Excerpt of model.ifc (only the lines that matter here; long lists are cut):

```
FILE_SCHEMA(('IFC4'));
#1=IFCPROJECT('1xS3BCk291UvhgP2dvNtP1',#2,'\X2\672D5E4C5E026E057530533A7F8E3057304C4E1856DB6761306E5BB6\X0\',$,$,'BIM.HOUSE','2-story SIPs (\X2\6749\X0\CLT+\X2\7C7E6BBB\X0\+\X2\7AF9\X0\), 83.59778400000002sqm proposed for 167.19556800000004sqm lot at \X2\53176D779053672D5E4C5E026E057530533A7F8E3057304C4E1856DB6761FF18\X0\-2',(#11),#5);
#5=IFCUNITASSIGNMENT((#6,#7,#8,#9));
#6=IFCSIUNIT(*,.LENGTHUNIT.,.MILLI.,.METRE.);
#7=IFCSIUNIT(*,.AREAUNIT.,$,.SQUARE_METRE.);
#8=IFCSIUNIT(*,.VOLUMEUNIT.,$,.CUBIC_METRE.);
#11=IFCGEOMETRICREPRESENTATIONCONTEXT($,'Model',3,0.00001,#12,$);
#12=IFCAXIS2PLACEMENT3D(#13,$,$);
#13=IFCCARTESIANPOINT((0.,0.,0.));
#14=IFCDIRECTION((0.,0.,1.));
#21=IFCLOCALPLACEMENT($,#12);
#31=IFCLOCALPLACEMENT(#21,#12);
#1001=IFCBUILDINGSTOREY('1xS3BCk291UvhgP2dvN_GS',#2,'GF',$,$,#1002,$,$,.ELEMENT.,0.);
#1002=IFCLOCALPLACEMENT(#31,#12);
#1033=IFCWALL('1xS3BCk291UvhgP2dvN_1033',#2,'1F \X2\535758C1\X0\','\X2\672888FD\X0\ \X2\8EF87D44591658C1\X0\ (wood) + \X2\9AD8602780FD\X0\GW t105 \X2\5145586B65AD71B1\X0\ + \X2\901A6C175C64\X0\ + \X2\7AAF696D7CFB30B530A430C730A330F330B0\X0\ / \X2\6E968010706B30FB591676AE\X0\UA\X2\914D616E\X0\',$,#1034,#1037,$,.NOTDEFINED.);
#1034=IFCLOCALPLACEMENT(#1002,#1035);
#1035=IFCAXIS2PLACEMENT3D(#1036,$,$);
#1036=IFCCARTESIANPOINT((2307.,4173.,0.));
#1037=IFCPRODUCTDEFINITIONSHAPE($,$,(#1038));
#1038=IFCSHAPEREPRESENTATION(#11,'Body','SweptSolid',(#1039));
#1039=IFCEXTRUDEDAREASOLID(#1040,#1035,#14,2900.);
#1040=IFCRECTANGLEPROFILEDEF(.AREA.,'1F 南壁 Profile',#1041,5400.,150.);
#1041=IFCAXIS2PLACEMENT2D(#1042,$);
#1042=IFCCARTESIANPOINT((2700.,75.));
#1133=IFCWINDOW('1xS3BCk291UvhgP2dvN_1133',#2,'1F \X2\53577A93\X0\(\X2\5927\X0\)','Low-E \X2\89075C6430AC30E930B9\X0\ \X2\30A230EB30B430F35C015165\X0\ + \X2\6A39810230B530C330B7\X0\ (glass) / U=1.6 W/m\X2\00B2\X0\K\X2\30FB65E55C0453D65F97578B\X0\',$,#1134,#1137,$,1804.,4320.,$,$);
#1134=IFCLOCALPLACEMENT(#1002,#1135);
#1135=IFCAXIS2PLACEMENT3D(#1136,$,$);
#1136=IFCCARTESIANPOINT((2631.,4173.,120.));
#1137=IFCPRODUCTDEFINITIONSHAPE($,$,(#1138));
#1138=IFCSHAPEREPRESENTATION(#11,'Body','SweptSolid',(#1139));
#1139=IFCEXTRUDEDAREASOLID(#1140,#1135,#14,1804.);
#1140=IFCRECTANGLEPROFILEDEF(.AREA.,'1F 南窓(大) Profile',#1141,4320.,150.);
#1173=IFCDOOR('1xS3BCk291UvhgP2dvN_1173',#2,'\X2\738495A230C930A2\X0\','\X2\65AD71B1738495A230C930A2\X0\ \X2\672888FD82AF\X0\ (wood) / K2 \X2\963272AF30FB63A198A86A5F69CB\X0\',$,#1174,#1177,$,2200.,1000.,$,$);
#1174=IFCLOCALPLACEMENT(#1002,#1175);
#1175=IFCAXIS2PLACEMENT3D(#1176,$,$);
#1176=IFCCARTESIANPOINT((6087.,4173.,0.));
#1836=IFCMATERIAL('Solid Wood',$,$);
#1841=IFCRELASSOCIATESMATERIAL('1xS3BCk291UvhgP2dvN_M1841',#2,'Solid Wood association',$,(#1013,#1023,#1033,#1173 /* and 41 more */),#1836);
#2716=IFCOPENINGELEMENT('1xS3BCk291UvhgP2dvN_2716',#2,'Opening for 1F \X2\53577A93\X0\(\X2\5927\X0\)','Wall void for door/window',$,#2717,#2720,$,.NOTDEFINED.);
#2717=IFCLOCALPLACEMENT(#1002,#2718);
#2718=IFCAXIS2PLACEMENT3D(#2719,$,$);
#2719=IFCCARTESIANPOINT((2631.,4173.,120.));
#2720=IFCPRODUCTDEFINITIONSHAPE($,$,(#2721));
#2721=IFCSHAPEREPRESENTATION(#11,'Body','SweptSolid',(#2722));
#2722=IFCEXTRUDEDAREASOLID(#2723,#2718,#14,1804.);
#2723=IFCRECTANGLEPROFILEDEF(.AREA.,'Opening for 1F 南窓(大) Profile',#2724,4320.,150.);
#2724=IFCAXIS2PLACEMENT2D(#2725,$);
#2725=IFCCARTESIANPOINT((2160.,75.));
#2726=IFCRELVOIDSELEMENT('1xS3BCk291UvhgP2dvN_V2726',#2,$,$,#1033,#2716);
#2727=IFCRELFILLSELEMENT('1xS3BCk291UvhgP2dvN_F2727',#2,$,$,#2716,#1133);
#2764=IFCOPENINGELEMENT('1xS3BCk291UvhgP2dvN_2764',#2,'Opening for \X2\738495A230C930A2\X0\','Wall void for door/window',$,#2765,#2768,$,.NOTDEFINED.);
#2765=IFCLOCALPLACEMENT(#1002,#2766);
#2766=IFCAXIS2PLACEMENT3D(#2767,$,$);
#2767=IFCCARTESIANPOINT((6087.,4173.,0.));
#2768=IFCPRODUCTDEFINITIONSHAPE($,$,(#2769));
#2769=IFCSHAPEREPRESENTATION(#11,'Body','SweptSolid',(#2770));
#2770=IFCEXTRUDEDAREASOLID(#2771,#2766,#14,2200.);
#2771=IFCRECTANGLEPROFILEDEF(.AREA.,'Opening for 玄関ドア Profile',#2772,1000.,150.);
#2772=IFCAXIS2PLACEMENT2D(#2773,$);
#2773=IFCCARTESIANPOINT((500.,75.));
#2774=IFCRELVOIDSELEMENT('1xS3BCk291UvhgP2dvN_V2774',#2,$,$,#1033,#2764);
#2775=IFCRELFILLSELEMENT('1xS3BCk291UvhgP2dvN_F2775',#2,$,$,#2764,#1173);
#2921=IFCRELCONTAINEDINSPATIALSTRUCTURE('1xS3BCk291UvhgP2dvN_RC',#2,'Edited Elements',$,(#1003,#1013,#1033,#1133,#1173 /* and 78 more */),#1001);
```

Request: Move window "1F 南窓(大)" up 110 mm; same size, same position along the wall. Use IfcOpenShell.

```python
import numpy as np
import ifcopenshell
import ifcopenshell.api.geometry
import ifcopenshell.util.placement
import ifcopenshell.util.unit

model = ifcopenshell.open("model.ifc")
unit_scale = ifcopenshell.util.unit.calculate_unit_scale(model)

window = model.by_guid("1xS3BCk291UvhgP2dvN_1133")
opening = window.FillsVoids[0].RelatingOpeningElement
dz = 0.11 / unit_scale

shift = np.array([0.0, 0.0, dz])
# The window is not placed relative to its opening, so move both.
for product in (opening, window):
    matrix = ifcopenshell.util.placement.get_local_placement(product.ObjectPlacement)
    matrix[:3, 3] += shift
    ifcopenshell.api.geometry.edit_object_placement(model, product=product, matrix=matrix, is_si=False)

print(f"moved by {dz * unit_scale:+.3f} m")

model.write("model_rev.ifc")
```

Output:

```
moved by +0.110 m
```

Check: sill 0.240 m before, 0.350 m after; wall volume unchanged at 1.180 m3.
